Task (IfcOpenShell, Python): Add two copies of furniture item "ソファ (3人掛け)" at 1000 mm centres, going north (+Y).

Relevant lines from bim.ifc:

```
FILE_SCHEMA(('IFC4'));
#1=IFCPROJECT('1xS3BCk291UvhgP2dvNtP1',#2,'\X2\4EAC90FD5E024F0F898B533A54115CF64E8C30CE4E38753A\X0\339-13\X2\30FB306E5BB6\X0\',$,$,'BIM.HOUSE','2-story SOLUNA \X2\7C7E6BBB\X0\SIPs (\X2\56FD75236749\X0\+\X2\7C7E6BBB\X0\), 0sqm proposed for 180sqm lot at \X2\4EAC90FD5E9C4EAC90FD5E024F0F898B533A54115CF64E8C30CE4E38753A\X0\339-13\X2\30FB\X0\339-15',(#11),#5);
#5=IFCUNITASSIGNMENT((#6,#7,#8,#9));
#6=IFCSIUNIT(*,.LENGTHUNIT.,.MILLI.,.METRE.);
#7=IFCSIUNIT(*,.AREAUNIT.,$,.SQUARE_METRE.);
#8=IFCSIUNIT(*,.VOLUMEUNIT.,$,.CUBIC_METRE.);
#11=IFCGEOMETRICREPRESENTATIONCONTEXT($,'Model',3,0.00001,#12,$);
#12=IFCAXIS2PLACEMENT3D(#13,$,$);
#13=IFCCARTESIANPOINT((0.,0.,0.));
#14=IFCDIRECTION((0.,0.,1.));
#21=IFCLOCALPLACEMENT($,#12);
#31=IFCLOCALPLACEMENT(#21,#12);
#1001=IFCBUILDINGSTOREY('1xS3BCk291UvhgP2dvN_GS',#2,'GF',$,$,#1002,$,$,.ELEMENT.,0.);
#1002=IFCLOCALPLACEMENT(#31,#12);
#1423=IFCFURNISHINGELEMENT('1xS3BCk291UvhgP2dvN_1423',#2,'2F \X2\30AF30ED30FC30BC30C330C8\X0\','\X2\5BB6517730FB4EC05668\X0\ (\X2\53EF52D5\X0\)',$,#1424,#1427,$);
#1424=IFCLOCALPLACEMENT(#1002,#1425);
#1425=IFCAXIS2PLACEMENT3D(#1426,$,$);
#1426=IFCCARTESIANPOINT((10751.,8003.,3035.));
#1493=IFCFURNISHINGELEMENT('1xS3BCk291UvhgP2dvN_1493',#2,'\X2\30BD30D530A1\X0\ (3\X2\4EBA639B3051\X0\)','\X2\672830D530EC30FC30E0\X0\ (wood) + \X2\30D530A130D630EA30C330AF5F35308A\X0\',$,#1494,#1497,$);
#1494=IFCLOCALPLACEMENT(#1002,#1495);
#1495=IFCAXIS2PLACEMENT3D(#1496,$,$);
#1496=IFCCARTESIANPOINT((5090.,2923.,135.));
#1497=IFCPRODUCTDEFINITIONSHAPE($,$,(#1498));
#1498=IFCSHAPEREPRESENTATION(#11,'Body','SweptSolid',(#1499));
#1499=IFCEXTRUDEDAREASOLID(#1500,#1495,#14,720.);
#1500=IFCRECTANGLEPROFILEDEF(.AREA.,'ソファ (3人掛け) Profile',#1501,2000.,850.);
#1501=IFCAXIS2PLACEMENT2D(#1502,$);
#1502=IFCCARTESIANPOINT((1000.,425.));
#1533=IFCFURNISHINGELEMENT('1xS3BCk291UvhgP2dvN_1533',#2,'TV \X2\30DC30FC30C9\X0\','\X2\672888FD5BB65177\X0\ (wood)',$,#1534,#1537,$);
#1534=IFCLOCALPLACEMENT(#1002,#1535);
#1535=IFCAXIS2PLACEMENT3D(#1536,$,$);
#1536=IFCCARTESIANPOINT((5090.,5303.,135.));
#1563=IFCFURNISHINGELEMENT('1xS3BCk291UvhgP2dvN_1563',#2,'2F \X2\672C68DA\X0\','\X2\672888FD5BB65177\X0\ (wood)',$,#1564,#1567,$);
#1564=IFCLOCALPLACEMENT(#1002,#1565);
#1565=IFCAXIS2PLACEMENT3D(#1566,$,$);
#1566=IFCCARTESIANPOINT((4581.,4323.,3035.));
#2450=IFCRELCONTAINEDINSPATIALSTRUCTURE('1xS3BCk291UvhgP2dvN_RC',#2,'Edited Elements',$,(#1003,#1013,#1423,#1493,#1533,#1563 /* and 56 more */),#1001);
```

```python
import numpy as np
import ifcopenshell
import ifcopenshell.api.geometry
import ifcopenshell.api.root
import ifcopenshell.util.element
import ifcopenshell.util.placement
import ifcopenshell.util.unit

model = ifcopenshell.open("bim.ifc")
unit_scale = ifcopenshell.util.unit.calculate_unit_scale(model)


def reuse_history(source, copy):
    """copy_class also copies each property set's owner history, people and application; keep the originals."""
    for rel in copy.IsDefinedBy:
        if rel.is_a("IfcRelDefinesByProperties") and (history := rel.RelatingPropertyDefinition.OwnerHistory):
            rel.RelatingPropertyDefinition.OwnerHistory = source.OwnerHistory
            ifcopenshell.util.element.remove_deep2(model, history)


source = model.by_guid("1xS3BCk291UvhgP2dvN_1493")
base = ifcopenshell.util.placement.get_local_placement(source.ObjectPlacement)
step = np.array([0.0, 1.0, 0.0]) * 1 / unit_scale

for i in range(1, 3):
    copy = ifcopenshell.api.root.copy_class(model, product=source)
    copy.Representation = ifcopenshell.util.element.copy_deep(
        model, source.Representation, exclude=["IfcGeometricRepresentationContext", "IfcRepresentationMap"]
    )
    reuse_history(source, copy)
    matrix = base.copy()
    matrix[:3, 3] += i * step
    print("added at", matrix[:3, 3].round(3) + 0.0)
    ifcopenshell.api.geometry.edit_object_placement(model, product=copy, matrix=matrix, is_si=False)

model.write("bim_v2.ifc")
```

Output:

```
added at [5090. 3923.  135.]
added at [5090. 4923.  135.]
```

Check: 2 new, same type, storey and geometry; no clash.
